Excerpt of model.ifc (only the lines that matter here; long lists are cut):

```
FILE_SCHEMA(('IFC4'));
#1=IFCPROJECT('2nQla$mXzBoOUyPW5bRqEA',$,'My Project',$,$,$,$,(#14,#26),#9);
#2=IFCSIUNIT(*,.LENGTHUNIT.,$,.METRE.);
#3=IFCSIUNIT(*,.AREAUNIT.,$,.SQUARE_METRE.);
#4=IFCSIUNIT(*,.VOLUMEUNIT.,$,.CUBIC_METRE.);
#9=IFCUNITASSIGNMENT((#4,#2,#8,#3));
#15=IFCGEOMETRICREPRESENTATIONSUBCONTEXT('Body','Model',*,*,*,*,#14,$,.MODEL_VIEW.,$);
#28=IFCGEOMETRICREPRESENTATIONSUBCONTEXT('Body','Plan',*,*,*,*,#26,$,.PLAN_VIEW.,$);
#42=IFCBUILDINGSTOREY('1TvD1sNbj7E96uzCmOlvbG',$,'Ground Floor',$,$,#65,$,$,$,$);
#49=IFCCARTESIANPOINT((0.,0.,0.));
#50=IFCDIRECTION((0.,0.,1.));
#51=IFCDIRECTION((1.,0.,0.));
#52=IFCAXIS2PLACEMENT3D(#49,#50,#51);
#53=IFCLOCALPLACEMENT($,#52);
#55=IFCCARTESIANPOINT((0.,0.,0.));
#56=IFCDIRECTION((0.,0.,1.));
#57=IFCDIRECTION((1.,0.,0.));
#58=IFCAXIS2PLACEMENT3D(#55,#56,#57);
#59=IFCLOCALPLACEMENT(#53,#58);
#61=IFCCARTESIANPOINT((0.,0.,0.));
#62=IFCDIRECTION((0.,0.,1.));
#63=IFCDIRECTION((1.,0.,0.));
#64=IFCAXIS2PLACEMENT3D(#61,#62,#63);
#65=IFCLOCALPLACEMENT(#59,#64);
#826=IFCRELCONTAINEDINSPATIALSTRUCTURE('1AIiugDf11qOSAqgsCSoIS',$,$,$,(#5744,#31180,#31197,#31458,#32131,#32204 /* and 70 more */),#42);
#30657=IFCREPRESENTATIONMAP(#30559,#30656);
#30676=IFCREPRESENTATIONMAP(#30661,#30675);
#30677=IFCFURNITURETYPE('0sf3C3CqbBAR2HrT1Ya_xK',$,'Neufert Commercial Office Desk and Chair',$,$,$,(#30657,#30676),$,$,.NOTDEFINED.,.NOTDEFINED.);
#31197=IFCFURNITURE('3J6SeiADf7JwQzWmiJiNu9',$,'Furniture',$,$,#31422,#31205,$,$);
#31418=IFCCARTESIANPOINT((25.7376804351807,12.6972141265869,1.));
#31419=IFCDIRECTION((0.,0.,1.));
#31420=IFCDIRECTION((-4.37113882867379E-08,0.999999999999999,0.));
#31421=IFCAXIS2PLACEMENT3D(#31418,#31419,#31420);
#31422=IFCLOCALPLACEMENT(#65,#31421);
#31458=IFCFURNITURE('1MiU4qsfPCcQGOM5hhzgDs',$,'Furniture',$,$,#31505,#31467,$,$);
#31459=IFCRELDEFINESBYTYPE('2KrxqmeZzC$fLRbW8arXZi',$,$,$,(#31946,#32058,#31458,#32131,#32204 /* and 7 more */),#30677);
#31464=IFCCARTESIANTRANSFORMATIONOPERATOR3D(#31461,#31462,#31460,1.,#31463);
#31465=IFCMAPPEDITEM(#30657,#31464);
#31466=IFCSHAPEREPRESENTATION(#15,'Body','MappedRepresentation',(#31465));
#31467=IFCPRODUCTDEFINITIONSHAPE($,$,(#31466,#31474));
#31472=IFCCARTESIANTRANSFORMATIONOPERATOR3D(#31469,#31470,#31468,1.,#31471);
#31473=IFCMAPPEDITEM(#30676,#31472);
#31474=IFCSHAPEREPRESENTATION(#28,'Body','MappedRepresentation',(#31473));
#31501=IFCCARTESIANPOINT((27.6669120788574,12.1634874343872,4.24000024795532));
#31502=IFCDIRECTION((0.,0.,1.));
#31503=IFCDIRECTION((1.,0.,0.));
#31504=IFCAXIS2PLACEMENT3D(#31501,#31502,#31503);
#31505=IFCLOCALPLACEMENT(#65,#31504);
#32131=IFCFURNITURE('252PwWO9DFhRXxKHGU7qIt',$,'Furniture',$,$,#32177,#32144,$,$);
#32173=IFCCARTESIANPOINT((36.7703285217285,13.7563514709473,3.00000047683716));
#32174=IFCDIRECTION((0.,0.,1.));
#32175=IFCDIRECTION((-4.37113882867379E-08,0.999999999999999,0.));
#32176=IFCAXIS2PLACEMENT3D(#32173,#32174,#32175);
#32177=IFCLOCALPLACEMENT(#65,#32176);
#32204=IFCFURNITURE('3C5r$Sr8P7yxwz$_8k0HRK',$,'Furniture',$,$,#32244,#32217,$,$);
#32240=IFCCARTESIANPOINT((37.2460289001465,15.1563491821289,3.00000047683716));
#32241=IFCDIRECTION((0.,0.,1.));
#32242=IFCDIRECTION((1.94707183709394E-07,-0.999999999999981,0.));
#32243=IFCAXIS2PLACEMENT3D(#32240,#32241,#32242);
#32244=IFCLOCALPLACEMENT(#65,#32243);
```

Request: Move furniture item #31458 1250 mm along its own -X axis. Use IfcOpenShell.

```python
import ifcopenshell
import ifcopenshell.api.geometry
import ifcopenshell.util.placement
import ifcopenshell.util.unit

model = ifcopenshell.open("model.ifc")
unit_scale = ifcopenshell.util.unit.calculate_unit_scale(model)

item = model.by_id(31458)
matrix = ifcopenshell.util.placement.get_local_placement(item.ObjectPlacement)
matrix[:3, 3] -= matrix[:3, 0] * 1.25 / unit_scale
ifcopenshell.api.geometry.edit_object_placement(model, product=item, matrix=matrix, is_si=False)

print(ifcopenshell.util.placement.get_local_placement(item.ObjectPlacement).round(3) + 0.0)

model.write("model-out.ifc")
```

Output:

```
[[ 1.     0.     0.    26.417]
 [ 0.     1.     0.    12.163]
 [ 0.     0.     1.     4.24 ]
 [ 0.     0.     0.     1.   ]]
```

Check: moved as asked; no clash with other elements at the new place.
